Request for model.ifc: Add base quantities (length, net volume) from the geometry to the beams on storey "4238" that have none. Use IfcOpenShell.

First a look at what the model holds.

```python
import ifcopenshell
import ifcopenshell.util.element
import ifcopenshell.util.unit

model = ifcopenshell.open("model.ifc")
print(model.schema)
for unit_type in ("LENGTHUNIT", "AREAUNIT", "VOLUMEUNIT"):
    print(unit_type, ifcopenshell.util.unit.calculate_unit_scale(model, unit_type))
storey = next(s for s in model.by_type("IfcBuildingStorey") if s.Name == "4238")
beams = [e for e in ifcopenshell.util.element.get_decomposition(storey) if e.is_a("IfcBeam")]
for e in sorted(beams, key=lambda e: e.id()):
    print(e.id(), e.is_a(), e.Name, list(ifcopenshell.util.element.get_psets(e, qtos_only=True)), sep=" | ")
```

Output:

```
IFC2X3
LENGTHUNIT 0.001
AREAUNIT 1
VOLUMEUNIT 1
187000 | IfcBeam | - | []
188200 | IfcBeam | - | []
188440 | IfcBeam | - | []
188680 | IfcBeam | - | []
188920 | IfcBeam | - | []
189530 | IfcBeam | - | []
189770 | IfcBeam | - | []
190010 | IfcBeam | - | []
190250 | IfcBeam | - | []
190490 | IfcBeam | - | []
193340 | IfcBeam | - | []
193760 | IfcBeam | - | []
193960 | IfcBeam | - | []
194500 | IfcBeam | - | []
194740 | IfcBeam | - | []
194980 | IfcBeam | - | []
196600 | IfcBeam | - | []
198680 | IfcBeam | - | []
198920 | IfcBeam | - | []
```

```python
import ifcopenshell
import ifcopenshell.api.pset
import ifcopenshell.geom
import ifcopenshell.util.element
import ifcopenshell.util.shape
import ifcopenshell.util.unit

model = ifcopenshell.open("model.ifc")
unit_scale = ifcopenshell.util.unit.calculate_unit_scale(model)
volume_scale = ifcopenshell.util.unit.calculate_unit_scale(model, "VOLUMEUNIT")
settings = ifcopenshell.geom.settings()

storey = next(s for s in model.by_type("IfcBuildingStorey") if s.Name == "4238")
beams = [e for e in ifcopenshell.util.element.get_decomposition(storey) if e.is_a("IfcBeam")]

for e in sorted(beams, key=lambda e: e.id()):
    if ifcopenshell.util.element.get_psets(e, qtos_only=True, should_inherit=False):
        continue
    # Geometry comes back in metres, in the element's own axes.
    shape = ifcopenshell.geom.create_shape(settings, e)
    values = {
        "Length": ifcopenshell.util.shape.get_max_xyz(shape.geometry) / unit_scale,
        "NetVolume": ifcopenshell.util.shape.get_volume(shape.geometry) / volume_scale,
    }
    qto = ifcopenshell.api.pset.add_qto(model, product=e, name="BaseQuantities")
    ifcopenshell.api.pset.edit_qto(model, qto=qto, properties=values)
    print(e.id(), {k: round(v, 3) for k, v in values.items()})

model.write("model_rev.ifc")
```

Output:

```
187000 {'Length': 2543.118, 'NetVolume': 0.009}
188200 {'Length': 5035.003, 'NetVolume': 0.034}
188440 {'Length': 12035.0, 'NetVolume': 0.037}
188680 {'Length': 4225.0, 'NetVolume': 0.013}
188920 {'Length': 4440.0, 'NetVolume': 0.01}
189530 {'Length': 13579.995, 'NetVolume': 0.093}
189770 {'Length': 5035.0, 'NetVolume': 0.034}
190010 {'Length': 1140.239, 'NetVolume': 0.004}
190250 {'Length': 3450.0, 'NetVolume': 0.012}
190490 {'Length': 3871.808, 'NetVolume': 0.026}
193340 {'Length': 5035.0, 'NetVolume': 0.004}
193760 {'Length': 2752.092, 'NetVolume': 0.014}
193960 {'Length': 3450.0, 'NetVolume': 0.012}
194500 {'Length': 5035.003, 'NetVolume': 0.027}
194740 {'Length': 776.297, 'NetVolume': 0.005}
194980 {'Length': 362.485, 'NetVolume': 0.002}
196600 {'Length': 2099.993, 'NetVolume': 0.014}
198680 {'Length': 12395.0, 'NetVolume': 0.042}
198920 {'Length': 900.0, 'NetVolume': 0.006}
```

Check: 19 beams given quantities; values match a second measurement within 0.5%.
